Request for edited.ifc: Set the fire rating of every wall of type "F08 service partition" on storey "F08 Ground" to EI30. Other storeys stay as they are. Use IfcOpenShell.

First a look at what the model holds.

```python
import ifcopenshell
import ifcopenshell.util.element

model = ifcopenshell.open("edited.ifc")
print(model.schema)
storey = next(s for s in model.by_type("IfcBuildingStorey") if s.Name == "F08 Ground")
walls = [e for e in ifcopenshell.util.element.get_decomposition(storey) if e.is_a("IfcWall")]
seen = {}
for e in walls:
    element_type = ifcopenshell.util.element.get_type(e)
    key = (element_type.Name if element_type != e and element_type else None, ifcopenshell.util.element.get_pset(e, "Pset_WallCommon", "FireRating"))
    seen[key] = seen.get(key, 0) + 1
for (name, value), count in sorted(seen.items(), key=str):
    print(count, "x", name, "|", value)
```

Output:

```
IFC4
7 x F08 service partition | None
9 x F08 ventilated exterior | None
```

```python
import ifcopenshell
import ifcopenshell.api.pset
import ifcopenshell.util.element

model = ifcopenshell.open("edited.ifc")

storey = next(s for s in model.by_type("IfcBuildingStorey") if s.Name == "F08 Ground")
walls = [e for e in ifcopenshell.util.element.get_decomposition(storey) if e.is_a("IfcWall")]

count = 0
for e in walls:
    element_type = ifcopenshell.util.element.get_type(e)
    if element_type in (None, e) or element_type.Name != "F08 service partition":
        continue
    # add_pset returns the element's existing set when there is one.
    pset = ifcopenshell.api.pset.add_pset(model, product=e, name="Pset_WallCommon")
    ifcopenshell.api.pset.edit_pset(model, pset=pset, properties={"FireRating": "EI30"})
    count += 1

print(count, "walls updated")

model.write("edited_edited.ifc")
```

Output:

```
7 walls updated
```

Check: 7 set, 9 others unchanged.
